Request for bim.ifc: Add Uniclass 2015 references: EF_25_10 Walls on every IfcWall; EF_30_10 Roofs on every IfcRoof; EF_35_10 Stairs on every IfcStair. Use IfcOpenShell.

First a look at what the model holds.

```python
import ifcopenshell

model = ifcopenshell.open("bim.ifc")
print(model.schema)
print("classifications:", [c.Name for c in model.by_type("IfcClassification")])
for ifc_class in ("IfcDoor", "IfcRoof", "IfcStair", "IfcWall", "IfcWindow"):
    print(ifc_class, len(model.by_type(ifc_class)))
```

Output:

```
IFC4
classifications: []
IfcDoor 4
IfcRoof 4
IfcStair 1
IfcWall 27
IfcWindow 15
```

```python
import ifcopenshell
import ifcopenshell.api.classification

model = ifcopenshell.open("bim.ifc")

system = ifcopenshell.api.classification.add_classification(model, classification="Uniclass 2015")

codes = {
    "IfcWall": ("EF_25_10", "Walls"),
    "IfcRoof": ("EF_30_10", "Roofs"),
    "IfcStair": ("EF_35_10", "Stairs"),
}
for ifc_class, (code, name) in codes.items():
    products = model.by_type(ifc_class)
    ifcopenshell.api.classification.add_reference(
        model, products=products, classification=system, identification=code, name=name
    )
    print(code, len(products))

model.write("bim-out.ifc")
```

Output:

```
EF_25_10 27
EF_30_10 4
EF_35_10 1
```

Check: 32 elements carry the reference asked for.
